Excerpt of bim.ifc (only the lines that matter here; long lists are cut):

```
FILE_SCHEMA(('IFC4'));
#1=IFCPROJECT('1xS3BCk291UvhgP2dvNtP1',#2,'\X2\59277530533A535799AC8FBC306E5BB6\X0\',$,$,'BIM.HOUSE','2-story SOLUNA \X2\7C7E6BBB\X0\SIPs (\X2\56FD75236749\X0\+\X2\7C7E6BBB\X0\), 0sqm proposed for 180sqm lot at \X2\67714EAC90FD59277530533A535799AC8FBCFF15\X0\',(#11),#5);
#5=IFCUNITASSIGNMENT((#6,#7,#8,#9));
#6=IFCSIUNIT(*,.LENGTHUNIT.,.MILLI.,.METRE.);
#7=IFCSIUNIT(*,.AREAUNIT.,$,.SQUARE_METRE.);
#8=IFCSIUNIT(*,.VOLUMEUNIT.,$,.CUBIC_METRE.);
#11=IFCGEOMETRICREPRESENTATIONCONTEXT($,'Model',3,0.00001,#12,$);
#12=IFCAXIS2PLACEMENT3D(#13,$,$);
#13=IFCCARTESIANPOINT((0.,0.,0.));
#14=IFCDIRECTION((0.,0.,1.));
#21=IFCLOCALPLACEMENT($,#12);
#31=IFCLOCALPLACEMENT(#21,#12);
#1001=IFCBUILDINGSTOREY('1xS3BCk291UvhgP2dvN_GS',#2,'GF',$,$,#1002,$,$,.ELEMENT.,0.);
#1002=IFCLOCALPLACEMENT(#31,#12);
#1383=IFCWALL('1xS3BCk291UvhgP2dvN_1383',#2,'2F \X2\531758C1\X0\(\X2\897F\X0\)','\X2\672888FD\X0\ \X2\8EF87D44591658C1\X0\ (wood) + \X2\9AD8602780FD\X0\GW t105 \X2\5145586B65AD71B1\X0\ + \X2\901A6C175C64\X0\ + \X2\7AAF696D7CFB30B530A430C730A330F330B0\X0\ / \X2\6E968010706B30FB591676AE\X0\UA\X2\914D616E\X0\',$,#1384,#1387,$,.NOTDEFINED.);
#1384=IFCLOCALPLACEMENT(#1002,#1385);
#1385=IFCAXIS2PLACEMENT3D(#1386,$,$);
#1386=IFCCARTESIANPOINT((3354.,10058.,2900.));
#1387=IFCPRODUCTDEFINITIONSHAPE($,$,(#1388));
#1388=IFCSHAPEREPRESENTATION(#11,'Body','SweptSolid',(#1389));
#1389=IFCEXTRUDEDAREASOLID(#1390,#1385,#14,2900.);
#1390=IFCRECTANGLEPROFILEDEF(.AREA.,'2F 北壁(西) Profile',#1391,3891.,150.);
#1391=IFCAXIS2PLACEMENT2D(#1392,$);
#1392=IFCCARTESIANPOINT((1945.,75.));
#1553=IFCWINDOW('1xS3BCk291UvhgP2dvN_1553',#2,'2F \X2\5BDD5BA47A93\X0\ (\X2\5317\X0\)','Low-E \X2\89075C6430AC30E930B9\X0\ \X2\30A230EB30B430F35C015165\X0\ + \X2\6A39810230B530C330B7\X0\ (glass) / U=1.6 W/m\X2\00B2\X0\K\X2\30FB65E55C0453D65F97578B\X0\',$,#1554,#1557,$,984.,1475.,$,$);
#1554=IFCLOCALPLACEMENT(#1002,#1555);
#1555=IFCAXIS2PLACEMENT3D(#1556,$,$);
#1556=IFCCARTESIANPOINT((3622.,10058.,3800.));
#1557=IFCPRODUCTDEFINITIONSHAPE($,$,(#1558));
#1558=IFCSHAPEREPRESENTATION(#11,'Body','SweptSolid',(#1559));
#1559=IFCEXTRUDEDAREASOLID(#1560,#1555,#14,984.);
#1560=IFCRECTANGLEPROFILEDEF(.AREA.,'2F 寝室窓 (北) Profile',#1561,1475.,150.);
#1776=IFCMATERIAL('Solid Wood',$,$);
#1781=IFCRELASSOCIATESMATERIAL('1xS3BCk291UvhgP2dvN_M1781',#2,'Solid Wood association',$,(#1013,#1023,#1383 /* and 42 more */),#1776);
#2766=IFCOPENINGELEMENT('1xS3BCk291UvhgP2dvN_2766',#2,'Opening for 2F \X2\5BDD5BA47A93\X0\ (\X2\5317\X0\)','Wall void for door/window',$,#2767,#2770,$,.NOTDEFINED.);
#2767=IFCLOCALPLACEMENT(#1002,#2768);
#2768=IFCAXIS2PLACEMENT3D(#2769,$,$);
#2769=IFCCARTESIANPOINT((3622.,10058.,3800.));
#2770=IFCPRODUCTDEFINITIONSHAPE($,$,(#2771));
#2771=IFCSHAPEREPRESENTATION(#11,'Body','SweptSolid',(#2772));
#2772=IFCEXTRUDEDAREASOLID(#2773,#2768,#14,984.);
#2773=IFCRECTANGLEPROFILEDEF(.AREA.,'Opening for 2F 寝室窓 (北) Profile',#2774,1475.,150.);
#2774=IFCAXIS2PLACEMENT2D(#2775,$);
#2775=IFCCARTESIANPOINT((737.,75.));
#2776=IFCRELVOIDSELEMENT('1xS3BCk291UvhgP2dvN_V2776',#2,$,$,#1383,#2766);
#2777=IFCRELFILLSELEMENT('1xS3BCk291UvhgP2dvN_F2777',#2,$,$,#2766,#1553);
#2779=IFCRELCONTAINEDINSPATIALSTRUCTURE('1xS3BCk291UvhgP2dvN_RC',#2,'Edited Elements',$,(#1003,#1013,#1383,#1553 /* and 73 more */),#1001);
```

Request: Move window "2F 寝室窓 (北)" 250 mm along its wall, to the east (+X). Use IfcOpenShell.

```python
import ifcopenshell
import ifcopenshell.api.geometry
import ifcopenshell.util.placement
import ifcopenshell.util.unit

model = ifcopenshell.open("bim.ifc")
unit_scale = ifcopenshell.util.unit.calculate_unit_scale(model)

window = model.by_guid("1xS3BCk291UvhgP2dvN_1553")
opening = window.FillsVoids[0].RelatingOpeningElement
wall = opening.VoidsElements[0].RelatingBuildingElement

wall_matrix = ifcopenshell.util.placement.get_local_placement(wall.ObjectPlacement)
shift = wall_matrix[:3, 0] * 0.25 / unit_scale
before = ifcopenshell.util.placement.get_local_placement(window.ObjectPlacement)[:3, 3].copy()

# The window is not placed relative to its opening, so move both.
for product in (opening, window):
    matrix = ifcopenshell.util.placement.get_local_placement(product.ObjectPlacement)
    matrix[:3, 3] += shift
    ifcopenshell.api.geometry.edit_object_placement(model, product=product, matrix=matrix, is_si=False)

after = ifcopenshell.util.placement.get_local_placement(window.ObjectPlacement)[:3, 3]
print("window moved by", (after - before).round(3) + 0.0)

model.write("bim_edited.ifc")
```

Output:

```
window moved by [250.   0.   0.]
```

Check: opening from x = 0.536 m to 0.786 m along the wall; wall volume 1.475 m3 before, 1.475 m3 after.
